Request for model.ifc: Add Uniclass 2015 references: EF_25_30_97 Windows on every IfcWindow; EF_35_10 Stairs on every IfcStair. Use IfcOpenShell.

First a look at what the model holds.

```python
import ifcopenshell

model = ifcopenshell.open("model.ifc")
print(model.schema)
print("classifications:", [c.Name for c in model.by_type("IfcClassification")])
for ifc_class in ("IfcDoor", "IfcRoof", "IfcStair", "IfcWall", "IfcWindow"):
    print(ifc_class, len(model.by_type(ifc_class)))
```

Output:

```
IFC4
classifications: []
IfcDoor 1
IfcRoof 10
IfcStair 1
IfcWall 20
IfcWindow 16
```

```python
import ifcopenshell
import ifcopenshell.api.classification

model = ifcopenshell.open("model.ifc")

system = ifcopenshell.api.classification.add_classification(model, classification="Uniclass 2015")

codes = {
    "IfcWindow": ("EF_25_30_97", "Windows"),
    "IfcStair": ("EF_35_10", "Stairs"),
}
for ifc_class, (code, name) in codes.items():
    products = model.by_type(ifc_class)
    ifcopenshell.api.classification.add_reference(
        model, products=products, classification=system, identification=code, name=name
    )
    print(code, len(products))

model.write("model-out.ifc")
```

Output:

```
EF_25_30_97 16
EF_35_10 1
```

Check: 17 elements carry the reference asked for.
